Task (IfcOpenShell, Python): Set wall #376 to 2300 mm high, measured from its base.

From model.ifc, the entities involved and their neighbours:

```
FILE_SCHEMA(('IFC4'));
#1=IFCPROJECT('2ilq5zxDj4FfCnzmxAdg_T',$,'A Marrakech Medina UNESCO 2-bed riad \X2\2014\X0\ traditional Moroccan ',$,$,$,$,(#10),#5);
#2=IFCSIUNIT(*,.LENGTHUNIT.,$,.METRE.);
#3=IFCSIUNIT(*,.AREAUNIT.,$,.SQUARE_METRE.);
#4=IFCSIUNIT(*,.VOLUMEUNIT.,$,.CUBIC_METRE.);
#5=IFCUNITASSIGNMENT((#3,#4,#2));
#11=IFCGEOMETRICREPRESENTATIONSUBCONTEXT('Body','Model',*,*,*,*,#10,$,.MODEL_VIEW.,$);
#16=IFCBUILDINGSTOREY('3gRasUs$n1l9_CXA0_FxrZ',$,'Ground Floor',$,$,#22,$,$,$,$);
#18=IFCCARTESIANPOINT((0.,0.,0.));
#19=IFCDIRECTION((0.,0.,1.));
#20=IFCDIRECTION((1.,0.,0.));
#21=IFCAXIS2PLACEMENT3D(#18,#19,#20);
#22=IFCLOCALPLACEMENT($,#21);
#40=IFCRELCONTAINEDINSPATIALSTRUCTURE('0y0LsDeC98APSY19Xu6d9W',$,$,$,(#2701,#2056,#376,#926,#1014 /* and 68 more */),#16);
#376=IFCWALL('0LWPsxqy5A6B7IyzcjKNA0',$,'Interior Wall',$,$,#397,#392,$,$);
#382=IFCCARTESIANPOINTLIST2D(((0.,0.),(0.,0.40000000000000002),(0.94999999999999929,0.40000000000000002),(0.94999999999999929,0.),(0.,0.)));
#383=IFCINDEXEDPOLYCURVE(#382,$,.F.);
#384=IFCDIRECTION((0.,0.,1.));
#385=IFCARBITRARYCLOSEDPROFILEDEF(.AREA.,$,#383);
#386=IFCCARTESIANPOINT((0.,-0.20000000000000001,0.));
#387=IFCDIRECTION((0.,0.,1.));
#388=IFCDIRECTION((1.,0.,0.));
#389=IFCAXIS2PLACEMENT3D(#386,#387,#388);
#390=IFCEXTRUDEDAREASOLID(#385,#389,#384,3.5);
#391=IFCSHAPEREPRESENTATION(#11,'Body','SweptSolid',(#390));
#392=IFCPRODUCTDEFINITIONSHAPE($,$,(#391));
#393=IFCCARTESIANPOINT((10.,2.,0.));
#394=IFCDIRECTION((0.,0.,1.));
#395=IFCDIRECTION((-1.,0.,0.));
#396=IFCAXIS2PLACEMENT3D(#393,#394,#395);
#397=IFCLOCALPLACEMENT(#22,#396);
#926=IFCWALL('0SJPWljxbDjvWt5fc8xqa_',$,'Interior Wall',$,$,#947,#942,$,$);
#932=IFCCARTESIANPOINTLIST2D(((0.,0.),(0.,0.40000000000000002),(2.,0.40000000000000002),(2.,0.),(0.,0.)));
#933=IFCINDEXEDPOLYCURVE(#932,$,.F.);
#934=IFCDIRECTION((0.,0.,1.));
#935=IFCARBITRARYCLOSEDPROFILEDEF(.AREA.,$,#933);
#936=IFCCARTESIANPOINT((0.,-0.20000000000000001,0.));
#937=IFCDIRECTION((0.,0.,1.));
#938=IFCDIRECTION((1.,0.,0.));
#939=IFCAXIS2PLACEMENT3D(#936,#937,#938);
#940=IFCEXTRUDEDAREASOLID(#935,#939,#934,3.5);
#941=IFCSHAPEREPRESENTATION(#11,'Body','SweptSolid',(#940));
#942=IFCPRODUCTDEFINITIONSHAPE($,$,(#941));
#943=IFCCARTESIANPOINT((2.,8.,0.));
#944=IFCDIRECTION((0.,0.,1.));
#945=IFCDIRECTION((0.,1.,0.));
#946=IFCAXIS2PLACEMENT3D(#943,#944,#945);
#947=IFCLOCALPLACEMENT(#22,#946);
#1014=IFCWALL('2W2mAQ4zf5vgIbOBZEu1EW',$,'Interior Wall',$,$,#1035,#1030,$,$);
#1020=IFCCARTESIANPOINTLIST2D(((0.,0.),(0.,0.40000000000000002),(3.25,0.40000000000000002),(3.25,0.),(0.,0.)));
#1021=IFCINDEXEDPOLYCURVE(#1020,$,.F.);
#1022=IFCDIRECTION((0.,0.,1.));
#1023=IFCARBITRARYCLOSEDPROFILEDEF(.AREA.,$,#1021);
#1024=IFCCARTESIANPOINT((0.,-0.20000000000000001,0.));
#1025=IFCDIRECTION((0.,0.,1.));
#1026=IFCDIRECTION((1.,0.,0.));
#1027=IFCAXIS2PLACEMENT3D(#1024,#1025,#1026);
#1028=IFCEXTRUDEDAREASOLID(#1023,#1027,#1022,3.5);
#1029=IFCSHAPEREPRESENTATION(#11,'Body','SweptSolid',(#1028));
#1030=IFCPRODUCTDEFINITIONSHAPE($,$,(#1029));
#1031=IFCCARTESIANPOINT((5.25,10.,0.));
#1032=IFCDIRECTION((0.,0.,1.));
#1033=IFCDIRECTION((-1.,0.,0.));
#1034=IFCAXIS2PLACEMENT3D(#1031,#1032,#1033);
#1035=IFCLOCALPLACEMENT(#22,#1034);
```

```python
import ifcopenshell
import ifcopenshell.geom
import ifcopenshell.util.representation
import ifcopenshell.util.shape

model = ifcopenshell.open("model.ifc")
settings = ifcopenshell.geom.settings()


def volume(element):
    """Net volume in cubic metres, openings subtracted."""
    shape = ifcopenshell.geom.create_shape(settings, element)
    return ifcopenshell.util.shape.get_volume(shape.geometry)


wall = model.by_guid("0LWPsxqy5A6B7IyzcjKNA0")
before = volume(wall)

body = ifcopenshell.util.representation.get_representation(wall, "Model", "Body")
solid = body.Items[0]
old_height = solid.Depth
solid.Depth = 2.3
after = volume(wall)

print(f"height {old_height:g} -> {solid.Depth:g}, volume {before:.3f} -> {after:.3f} m3")

model.write("model_updated.ifc")
```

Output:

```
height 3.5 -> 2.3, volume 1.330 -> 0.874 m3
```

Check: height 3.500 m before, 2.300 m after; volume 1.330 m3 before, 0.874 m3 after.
